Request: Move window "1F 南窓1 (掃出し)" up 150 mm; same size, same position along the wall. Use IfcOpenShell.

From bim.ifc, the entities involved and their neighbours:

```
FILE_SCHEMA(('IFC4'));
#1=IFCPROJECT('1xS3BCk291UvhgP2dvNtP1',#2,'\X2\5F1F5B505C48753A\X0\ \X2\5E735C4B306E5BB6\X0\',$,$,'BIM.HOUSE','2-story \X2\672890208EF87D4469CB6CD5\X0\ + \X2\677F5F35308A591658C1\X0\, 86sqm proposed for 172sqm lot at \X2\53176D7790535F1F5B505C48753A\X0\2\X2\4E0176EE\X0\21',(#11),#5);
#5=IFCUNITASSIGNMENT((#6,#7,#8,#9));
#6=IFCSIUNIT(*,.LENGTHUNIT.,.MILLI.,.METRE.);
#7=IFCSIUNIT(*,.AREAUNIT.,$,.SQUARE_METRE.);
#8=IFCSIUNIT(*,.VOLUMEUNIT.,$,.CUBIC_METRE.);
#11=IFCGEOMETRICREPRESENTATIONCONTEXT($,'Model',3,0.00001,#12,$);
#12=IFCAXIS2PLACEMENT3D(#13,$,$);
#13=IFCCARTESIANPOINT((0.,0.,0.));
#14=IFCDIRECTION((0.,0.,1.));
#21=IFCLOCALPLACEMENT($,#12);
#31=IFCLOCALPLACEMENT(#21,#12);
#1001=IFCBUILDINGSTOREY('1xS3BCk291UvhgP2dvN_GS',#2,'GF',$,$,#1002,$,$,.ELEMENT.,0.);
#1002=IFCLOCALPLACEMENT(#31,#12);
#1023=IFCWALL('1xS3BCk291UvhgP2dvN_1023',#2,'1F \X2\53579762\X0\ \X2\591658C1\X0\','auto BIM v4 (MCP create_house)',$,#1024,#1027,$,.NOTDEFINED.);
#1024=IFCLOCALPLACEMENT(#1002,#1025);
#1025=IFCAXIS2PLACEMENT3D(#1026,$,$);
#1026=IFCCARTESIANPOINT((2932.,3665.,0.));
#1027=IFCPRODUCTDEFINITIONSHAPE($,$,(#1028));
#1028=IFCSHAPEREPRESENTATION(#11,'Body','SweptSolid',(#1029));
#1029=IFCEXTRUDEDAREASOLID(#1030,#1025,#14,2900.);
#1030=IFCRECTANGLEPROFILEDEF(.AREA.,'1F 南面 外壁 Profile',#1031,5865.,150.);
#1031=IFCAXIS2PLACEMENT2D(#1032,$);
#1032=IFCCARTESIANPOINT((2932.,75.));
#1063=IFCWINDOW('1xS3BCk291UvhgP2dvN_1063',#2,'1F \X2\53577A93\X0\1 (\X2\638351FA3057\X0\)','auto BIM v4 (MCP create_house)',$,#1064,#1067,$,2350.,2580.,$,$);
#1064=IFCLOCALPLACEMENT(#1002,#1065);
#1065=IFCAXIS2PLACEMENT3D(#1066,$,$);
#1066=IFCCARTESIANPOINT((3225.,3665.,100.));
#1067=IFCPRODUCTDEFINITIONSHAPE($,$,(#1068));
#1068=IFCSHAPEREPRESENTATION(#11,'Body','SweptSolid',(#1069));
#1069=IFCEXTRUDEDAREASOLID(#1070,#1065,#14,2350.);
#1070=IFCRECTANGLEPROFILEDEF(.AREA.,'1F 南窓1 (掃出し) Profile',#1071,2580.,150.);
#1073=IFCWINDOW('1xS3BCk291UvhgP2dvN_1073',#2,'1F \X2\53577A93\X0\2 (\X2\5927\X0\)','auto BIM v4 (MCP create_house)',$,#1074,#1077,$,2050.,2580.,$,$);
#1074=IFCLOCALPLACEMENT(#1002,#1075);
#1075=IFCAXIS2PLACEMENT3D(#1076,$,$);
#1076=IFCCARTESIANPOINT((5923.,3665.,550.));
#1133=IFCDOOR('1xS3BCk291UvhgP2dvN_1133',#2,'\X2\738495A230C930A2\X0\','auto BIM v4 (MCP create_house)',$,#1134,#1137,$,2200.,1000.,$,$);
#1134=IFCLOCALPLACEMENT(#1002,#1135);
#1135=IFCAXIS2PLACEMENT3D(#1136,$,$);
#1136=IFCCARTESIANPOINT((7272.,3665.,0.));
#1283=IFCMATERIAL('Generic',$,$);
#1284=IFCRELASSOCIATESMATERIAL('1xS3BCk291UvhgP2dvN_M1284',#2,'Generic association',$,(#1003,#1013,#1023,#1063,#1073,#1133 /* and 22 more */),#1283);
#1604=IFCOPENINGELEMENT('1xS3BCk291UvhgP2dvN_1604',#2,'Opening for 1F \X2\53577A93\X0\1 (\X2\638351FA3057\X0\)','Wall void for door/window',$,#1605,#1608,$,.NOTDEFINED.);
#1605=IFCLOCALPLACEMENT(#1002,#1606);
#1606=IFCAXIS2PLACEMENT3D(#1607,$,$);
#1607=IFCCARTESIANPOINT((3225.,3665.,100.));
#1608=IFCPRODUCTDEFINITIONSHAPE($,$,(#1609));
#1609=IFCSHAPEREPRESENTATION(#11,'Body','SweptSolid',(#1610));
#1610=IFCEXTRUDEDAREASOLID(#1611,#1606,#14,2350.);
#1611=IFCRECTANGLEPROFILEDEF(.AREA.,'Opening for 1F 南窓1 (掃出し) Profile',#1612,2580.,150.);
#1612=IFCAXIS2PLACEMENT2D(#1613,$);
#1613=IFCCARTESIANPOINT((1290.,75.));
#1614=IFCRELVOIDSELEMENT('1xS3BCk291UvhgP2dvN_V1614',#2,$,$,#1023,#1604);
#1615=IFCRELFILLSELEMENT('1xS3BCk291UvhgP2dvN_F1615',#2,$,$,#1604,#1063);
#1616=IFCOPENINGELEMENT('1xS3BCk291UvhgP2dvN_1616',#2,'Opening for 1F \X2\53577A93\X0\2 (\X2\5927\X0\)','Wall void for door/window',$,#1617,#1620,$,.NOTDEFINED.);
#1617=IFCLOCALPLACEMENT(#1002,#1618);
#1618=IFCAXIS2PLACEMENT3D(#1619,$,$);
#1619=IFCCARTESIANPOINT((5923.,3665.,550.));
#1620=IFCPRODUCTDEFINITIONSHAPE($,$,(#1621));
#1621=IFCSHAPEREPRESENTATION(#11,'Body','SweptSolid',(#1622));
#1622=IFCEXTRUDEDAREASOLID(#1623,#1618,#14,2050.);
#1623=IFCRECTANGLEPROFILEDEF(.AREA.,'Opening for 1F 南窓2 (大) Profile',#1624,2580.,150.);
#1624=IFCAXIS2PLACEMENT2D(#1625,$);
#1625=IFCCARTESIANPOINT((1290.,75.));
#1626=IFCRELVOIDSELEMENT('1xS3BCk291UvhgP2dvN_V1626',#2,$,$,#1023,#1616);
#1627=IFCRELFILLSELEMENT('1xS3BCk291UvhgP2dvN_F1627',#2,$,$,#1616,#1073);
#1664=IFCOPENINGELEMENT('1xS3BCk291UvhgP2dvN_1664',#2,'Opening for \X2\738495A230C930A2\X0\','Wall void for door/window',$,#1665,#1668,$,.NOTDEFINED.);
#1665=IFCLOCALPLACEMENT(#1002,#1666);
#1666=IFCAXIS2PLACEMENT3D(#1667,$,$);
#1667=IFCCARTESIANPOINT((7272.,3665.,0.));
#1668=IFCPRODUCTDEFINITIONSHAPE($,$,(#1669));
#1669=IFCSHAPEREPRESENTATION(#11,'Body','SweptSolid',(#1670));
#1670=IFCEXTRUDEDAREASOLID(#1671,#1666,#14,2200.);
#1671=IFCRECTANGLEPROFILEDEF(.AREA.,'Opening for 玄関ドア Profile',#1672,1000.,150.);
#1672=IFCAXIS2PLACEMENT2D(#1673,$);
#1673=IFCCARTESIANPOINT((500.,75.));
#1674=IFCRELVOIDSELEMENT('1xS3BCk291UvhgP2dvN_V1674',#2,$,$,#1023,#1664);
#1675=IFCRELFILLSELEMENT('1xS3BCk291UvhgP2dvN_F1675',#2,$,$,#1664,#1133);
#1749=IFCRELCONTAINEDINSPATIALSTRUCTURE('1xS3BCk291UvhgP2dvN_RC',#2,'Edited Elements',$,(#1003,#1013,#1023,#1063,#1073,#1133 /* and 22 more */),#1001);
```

```python
import numpy as np
import ifcopenshell
import ifcopenshell.api.geometry
import ifcopenshell.util.placement
import ifcopenshell.util.unit

model = ifcopenshell.open("bim.ifc")
unit_scale = ifcopenshell.util.unit.calculate_unit_scale(model)

window = model.by_id(1063)
opening = window.FillsVoids[0].RelatingOpeningElement
dz = 150.0

shift = np.array([0.0, 0.0, dz])
# The window is not placed relative to its opening, so move both.
for product in (opening, window):
    matrix = ifcopenshell.util.placement.get_local_placement(product.ObjectPlacement)
    matrix[:3, 3] += shift
    ifcopenshell.api.geometry.edit_object_placement(model, product=product, matrix=matrix, is_si=False)

print(f"moved by {dz * unit_scale:+.3f} m")

model.write("bim-out.ifc")
```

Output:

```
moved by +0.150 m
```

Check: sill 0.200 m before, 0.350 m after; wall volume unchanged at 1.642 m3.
